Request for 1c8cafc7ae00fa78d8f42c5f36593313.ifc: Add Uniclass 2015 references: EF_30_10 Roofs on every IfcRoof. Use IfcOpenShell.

First a look at what the model holds.

```python
import ifcopenshell

model = ifcopenshell.open("1c8cafc7ae00fa78d8f42c5f36593313.ifc")
print(model.schema)
print("classifications:", [c.Name for c in model.by_type("IfcClassification")])
for ifc_class in ("IfcDoor", "IfcRoof", "IfcStair", "IfcWall", "IfcWindow"):
    print(ifc_class, len(model.by_type(ifc_class)))
```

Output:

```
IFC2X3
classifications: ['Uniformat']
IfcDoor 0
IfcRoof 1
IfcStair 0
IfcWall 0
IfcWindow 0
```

```python
import ifcopenshell
import ifcopenshell.api.classification

model = ifcopenshell.open("1c8cafc7ae00fa78d8f42c5f36593313.ifc")

# IFC2X3 requires Source and Edition and has no link from the project to the system.
system = model.create_entity("IfcClassification", Source="NBS", Edition="2015", Name="Uniclass 2015")

codes = {
    "IfcRoof": ("EF_30_10", "Roofs"),
}
for ifc_class, (code, name) in codes.items():
    products = model.by_type(ifc_class)
    ifcopenshell.api.classification.add_reference(
        model, products=products, classification=system, identification=code, name=name
    )
    print(code, len(products))

model.write("1c8cafc7ae00fa78d8f42c5f36593313_v2.ifc")
```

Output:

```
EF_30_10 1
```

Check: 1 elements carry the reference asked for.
